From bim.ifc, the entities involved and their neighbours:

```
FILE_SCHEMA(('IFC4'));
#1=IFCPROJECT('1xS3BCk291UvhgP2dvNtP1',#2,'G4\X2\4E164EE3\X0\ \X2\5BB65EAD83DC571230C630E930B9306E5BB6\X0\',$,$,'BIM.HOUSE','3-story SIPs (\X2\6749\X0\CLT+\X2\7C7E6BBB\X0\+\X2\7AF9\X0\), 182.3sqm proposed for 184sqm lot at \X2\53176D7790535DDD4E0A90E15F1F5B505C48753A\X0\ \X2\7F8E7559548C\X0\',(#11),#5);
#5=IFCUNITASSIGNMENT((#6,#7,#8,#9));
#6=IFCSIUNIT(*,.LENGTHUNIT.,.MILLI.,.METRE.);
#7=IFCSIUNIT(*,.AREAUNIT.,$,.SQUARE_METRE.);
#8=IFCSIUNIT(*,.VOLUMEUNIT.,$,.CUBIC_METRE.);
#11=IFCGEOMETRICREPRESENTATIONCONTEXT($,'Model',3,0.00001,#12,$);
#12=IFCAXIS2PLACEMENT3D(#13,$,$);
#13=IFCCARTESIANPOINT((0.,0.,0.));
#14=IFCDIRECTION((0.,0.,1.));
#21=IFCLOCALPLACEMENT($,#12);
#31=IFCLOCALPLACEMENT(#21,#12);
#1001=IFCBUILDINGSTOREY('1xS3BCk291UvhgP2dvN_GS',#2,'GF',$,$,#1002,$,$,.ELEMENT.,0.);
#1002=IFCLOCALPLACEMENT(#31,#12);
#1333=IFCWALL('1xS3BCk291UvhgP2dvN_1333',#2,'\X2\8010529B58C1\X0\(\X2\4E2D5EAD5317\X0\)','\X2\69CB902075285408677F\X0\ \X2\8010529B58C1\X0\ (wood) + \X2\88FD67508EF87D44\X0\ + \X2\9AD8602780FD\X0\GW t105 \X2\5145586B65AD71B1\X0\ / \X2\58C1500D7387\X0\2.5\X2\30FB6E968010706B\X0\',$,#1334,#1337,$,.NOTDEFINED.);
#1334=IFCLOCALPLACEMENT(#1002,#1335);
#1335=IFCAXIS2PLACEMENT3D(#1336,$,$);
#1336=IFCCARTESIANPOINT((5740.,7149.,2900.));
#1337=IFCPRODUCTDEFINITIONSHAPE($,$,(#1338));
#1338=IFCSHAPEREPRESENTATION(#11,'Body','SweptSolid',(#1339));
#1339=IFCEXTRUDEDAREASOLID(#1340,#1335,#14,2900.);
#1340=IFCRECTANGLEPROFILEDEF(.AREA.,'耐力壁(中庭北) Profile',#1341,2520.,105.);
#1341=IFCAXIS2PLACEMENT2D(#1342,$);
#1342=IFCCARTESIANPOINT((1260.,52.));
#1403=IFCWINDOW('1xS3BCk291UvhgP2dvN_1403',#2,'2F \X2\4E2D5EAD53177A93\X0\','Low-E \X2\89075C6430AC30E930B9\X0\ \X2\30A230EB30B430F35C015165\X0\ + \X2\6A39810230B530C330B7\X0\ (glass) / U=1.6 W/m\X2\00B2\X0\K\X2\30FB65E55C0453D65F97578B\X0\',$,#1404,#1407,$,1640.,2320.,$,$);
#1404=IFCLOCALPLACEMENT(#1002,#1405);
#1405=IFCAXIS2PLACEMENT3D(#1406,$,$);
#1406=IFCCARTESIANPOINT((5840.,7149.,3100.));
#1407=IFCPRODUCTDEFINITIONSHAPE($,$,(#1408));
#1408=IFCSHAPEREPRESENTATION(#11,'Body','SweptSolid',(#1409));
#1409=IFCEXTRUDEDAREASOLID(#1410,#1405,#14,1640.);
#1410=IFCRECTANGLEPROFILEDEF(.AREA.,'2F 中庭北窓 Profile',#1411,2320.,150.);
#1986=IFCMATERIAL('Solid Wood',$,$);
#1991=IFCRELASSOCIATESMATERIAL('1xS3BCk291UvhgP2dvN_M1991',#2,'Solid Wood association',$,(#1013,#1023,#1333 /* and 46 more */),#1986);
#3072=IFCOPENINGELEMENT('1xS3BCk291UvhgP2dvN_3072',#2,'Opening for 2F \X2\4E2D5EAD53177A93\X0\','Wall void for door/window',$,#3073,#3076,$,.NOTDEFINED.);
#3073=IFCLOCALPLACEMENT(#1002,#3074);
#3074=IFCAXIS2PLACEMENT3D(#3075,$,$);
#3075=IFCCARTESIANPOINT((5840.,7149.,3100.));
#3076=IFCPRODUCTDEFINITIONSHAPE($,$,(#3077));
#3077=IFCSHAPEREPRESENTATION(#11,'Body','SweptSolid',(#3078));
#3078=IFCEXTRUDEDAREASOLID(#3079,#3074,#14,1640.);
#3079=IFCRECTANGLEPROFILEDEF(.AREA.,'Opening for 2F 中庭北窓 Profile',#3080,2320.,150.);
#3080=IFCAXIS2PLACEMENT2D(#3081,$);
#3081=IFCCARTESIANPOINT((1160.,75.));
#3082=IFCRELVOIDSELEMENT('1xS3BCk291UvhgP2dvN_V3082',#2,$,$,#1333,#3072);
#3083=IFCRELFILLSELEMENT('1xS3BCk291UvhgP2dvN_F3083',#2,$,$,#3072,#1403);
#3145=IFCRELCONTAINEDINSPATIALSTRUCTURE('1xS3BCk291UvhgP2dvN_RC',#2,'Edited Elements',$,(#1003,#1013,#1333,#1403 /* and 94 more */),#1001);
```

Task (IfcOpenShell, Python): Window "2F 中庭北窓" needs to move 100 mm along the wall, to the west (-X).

```python
import ifcopenshell
import ifcopenshell.api.geometry
import ifcopenshell.util.placement
import ifcopenshell.util.unit

model = ifcopenshell.open("bim.ifc")
unit_scale = ifcopenshell.util.unit.calculate_unit_scale(model)

window = model.by_id(1403)
opening = window.FillsVoids[0].RelatingOpeningElement
wall = opening.VoidsElements[0].RelatingBuildingElement

wall_matrix = ifcopenshell.util.placement.get_local_placement(wall.ObjectPlacement)
shift = wall_matrix[:3, 0] * -0.1 / unit_scale
before = ifcopenshell.util.placement.get_local_placement(window.ObjectPlacement)[:3, 3].copy()

# The window is not placed relative to its opening, so move both.
for product in (opening, window):
    matrix = ifcopenshell.util.placement.get_local_placement(product.ObjectPlacement)
    matrix[:3, 3] += shift
    ifcopenshell.api.geometry.edit_object_placement(model, product=product, matrix=matrix, is_si=False)

after = ifcopenshell.util.placement.get_local_placement(window.ObjectPlacement)[:3, 3]
print("window moved by", (after - before).round(3) + 0.0)

model.write("bim_edited.ifc")
```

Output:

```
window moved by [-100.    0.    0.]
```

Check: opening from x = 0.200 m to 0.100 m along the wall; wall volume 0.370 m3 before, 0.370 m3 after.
